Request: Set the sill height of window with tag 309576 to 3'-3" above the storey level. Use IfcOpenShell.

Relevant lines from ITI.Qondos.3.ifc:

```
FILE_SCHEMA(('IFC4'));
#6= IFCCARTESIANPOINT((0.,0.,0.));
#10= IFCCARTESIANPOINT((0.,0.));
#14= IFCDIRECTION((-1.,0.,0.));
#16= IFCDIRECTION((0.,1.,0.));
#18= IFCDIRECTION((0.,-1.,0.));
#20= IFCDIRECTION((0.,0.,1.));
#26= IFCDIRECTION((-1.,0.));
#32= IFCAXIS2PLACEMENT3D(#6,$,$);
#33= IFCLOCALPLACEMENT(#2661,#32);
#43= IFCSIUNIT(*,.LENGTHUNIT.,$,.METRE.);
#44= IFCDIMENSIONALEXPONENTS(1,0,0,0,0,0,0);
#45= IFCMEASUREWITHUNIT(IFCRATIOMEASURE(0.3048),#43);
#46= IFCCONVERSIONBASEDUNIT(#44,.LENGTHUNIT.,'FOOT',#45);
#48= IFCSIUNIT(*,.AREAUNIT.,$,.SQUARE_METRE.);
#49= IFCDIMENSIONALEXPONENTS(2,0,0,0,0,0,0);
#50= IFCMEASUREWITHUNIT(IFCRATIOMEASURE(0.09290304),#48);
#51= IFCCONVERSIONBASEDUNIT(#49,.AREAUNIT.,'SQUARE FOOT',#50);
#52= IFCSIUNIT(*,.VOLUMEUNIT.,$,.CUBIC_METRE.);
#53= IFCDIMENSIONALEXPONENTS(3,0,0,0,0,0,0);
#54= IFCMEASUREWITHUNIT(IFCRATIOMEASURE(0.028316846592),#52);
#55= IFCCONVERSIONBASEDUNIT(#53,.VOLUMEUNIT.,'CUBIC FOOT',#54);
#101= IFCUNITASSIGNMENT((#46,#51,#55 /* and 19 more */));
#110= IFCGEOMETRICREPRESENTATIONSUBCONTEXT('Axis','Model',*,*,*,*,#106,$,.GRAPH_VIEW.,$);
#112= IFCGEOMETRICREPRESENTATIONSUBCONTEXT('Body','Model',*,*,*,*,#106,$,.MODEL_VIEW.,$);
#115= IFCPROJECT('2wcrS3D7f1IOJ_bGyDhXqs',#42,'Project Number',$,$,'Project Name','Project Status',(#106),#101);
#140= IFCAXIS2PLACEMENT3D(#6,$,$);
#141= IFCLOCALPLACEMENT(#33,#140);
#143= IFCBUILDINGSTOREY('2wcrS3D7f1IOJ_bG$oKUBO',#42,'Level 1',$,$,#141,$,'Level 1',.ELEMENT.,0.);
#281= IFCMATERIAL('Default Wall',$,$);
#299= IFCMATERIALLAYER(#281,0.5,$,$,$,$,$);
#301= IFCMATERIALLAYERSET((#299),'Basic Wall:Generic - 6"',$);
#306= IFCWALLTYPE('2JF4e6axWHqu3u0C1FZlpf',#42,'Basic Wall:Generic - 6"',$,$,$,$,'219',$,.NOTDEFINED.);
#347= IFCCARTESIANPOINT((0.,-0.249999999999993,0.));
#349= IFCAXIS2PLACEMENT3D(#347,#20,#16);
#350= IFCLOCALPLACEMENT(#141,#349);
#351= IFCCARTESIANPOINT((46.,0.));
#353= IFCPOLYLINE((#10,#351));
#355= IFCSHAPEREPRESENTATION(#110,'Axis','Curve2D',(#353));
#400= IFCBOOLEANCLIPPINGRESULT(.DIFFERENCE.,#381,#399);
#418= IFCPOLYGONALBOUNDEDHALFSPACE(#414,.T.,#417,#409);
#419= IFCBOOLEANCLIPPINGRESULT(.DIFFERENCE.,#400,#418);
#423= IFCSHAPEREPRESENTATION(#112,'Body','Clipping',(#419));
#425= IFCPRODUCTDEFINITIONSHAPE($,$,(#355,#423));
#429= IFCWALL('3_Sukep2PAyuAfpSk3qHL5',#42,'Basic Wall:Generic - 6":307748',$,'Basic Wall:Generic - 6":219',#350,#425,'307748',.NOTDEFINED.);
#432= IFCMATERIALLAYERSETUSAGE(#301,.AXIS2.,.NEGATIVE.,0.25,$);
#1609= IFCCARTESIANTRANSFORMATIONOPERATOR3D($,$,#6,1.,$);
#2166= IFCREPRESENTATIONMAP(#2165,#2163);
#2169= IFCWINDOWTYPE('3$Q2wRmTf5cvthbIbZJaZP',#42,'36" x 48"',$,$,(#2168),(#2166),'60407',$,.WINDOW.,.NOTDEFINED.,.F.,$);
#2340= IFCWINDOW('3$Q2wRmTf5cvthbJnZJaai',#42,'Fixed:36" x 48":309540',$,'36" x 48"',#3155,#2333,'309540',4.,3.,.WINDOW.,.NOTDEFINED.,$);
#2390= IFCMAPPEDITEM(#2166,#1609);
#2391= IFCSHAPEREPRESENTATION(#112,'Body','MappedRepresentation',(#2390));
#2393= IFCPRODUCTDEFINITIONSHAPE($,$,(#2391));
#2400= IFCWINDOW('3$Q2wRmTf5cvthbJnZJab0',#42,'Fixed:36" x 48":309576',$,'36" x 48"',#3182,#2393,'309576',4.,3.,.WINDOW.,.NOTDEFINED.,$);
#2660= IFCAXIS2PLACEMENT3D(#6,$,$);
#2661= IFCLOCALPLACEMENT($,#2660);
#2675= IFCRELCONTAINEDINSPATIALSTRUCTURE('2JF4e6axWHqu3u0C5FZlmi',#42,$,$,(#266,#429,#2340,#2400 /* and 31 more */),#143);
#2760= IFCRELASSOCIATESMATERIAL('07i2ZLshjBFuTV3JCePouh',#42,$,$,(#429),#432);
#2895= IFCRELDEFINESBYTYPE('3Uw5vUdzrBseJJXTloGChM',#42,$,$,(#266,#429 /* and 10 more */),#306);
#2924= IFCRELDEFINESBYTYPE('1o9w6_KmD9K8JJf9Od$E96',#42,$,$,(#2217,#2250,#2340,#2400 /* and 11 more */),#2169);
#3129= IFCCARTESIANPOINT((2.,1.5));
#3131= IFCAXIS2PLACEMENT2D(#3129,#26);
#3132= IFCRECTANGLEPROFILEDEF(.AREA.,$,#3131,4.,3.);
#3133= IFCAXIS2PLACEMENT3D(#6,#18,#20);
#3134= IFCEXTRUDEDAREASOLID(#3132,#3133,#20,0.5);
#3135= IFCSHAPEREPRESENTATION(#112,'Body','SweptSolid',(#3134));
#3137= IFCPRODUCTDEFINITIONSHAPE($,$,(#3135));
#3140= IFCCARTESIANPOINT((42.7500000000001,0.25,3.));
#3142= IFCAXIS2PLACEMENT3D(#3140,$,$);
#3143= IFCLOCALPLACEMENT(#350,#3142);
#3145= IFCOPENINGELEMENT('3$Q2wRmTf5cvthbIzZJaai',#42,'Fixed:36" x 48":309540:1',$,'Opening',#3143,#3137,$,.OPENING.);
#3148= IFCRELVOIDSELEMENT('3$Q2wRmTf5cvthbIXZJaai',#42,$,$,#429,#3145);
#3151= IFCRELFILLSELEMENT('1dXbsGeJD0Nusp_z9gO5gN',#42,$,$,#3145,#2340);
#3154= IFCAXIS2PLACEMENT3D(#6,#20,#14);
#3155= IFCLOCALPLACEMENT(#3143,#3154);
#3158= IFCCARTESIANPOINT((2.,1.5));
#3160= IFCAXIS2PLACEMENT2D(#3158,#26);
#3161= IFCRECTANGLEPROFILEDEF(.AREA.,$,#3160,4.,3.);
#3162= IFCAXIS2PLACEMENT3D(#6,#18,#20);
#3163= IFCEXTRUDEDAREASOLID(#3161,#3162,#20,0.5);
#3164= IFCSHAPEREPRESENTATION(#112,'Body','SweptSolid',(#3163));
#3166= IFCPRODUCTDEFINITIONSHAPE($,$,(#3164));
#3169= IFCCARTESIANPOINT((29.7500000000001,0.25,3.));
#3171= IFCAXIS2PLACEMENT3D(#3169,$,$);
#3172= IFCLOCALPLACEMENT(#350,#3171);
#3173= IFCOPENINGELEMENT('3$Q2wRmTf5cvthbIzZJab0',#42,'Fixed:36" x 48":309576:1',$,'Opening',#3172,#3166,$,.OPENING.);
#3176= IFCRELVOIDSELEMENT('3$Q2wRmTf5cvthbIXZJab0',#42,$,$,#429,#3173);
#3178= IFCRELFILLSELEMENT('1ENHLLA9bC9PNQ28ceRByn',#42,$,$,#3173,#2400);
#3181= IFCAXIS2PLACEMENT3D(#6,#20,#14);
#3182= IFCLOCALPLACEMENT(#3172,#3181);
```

```python
import numpy as np
import ifcopenshell
import ifcopenshell.api.geometry
import ifcopenshell.geom
import ifcopenshell.util.element
import ifcopenshell.util.placement
import ifcopenshell.util.shape
import ifcopenshell.util.unit

model = ifcopenshell.open("ITI.Qondos.3.ifc")
unit_scale = ifcopenshell.util.unit.calculate_unit_scale(model)

window = model.by_id(2400)
opening = window.FillsVoids[0].RelatingOpeningElement
storey = ifcopenshell.util.element.get_container(window, ifc_class="IfcBuildingStorey")
level = ifcopenshell.util.placement.get_local_placement(storey.ObjectPlacement)[2, 3]

# The opening's origin need not be at the sill, so measure its lowest point.
shape = ifcopenshell.geom.create_shape(ifcopenshell.geom.settings(), opening)
bottom = ifcopenshell.util.shape.get_shape_bottom_elevation(shape, shape.geometry) / unit_scale
dz = level + 39 * 0.0254 / unit_scale - bottom

shift = np.array([0.0, 0.0, dz])
# The window is placed relative to its opening, so it follows when the opening moves.
matrix = ifcopenshell.util.placement.get_local_placement(opening.ObjectPlacement)
matrix[:3, 3] += shift
ifcopenshell.api.geometry.edit_object_placement(
    model, product=opening, matrix=matrix, is_si=False, should_transform_children=True
)

print(f"moved by {dz * unit_scale:+.3f} m")

model.write("ITI.Qondos.3_edited.ifc")
```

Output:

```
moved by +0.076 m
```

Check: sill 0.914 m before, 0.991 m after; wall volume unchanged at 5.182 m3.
